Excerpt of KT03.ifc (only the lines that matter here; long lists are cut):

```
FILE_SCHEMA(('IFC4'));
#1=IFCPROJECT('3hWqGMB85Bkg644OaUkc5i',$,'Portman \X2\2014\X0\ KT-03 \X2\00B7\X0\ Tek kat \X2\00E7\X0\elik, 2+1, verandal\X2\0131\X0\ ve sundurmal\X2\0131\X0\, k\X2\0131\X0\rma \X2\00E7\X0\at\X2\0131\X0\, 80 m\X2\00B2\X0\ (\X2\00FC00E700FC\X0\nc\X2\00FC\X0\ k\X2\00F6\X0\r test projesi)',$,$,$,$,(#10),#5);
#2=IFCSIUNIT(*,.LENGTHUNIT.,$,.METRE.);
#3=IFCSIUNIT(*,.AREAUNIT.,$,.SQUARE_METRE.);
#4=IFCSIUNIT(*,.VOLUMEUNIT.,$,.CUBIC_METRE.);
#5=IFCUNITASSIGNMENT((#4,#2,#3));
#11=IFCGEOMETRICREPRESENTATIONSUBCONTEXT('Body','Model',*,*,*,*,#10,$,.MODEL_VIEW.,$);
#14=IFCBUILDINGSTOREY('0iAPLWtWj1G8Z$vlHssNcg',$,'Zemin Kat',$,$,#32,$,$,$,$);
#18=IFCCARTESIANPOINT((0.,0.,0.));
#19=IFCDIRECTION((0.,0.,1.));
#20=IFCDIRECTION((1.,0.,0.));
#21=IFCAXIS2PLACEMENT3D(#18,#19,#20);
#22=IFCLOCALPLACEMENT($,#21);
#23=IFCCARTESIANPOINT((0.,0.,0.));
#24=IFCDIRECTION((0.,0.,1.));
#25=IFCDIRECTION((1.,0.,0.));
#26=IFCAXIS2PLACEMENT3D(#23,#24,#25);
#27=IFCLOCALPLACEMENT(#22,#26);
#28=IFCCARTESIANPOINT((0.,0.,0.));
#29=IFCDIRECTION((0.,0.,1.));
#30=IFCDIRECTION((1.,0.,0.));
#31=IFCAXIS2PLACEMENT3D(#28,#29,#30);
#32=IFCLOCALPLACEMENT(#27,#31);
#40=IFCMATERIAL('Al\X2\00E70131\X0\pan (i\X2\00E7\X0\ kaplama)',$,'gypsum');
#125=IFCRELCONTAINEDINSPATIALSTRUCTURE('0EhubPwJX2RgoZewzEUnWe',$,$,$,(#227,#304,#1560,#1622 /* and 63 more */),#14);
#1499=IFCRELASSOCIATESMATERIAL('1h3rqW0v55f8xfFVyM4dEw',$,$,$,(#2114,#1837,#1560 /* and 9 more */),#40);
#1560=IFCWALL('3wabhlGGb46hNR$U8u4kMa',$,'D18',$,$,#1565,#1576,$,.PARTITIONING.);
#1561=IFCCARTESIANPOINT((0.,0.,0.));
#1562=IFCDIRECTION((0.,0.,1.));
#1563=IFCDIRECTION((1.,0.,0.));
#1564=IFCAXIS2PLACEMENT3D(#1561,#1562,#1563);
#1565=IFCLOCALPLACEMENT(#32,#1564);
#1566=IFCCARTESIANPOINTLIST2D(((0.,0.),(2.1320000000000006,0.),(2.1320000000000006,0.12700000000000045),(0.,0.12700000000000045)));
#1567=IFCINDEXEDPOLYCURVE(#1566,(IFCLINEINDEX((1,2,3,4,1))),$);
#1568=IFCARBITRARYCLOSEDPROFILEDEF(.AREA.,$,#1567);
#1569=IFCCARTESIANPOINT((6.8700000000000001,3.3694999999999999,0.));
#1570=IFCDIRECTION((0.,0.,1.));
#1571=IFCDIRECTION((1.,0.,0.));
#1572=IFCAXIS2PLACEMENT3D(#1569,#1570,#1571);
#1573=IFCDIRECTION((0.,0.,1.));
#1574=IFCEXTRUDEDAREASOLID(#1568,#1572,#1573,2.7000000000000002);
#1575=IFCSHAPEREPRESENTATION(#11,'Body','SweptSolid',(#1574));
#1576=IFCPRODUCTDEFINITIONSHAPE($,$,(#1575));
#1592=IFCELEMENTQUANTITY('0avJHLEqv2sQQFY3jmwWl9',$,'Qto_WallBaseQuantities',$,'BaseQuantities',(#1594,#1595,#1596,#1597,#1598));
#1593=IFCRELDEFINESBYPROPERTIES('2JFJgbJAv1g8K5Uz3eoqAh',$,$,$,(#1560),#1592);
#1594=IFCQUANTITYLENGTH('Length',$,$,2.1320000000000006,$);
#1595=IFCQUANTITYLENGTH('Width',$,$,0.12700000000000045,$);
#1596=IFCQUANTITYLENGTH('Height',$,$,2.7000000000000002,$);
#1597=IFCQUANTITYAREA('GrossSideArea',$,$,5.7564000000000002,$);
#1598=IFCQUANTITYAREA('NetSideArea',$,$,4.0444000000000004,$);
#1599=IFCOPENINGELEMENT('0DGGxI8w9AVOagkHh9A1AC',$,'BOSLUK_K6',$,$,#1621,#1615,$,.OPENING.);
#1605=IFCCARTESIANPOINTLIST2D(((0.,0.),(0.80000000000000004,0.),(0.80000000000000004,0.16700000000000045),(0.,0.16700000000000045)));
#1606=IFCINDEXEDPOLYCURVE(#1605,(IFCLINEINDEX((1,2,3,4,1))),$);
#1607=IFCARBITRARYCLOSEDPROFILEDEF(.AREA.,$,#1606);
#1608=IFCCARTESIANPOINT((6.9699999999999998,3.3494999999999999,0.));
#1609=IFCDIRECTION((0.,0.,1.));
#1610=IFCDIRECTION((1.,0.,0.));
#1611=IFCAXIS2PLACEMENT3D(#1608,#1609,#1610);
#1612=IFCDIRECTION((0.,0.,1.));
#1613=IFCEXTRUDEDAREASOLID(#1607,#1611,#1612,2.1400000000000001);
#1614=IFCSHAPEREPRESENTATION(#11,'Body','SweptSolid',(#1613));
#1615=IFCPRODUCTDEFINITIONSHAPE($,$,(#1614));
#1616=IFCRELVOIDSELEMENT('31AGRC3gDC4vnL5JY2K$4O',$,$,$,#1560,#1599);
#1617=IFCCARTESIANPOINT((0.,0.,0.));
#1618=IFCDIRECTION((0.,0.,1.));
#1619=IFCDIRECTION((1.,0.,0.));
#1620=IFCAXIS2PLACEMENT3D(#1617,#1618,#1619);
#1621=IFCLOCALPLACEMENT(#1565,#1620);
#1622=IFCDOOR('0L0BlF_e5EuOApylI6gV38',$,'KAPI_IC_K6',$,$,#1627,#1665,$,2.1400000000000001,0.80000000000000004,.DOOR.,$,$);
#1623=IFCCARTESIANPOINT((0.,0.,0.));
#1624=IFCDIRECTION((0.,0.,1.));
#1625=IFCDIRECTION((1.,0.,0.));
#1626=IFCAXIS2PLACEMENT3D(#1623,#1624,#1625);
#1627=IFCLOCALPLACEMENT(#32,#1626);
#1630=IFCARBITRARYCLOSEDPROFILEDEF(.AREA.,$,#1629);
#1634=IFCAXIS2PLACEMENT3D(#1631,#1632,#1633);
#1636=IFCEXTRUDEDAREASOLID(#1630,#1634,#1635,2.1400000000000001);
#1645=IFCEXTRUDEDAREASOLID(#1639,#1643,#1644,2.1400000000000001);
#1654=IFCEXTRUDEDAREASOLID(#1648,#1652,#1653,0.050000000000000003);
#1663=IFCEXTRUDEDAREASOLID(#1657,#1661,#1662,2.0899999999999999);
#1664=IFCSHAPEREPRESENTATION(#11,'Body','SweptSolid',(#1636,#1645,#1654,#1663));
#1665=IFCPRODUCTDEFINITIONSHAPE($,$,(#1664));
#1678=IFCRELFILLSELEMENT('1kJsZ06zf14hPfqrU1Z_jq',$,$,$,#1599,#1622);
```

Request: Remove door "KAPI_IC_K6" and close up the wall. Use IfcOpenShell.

```python
import ifcopenshell
import ifcopenshell.api.feature
import ifcopenshell.api.pset
import ifcopenshell.api.root
import ifcopenshell.geom
import ifcopenshell.util.element
import ifcopenshell.util.shape
import ifcopenshell.util.unit

model = ifcopenshell.open("KT03.ifc")
area_scale = ifcopenshell.util.unit.calculate_unit_scale(model, "AREAUNIT")
settings = ifcopenshell.geom.settings()


def volume(element):
    """Net volume in cubic metres, openings subtracted."""
    shape = ifcopenshell.geom.create_shape(settings, element)
    return ifcopenshell.util.shape.get_volume(shape.geometry)


door = model.by_guid("0L0BlF_e5EuOApylI6gV38")
opening = door.FillsVoids[0].RelatingOpeningElement
wall = opening.VoidsElements[0].RelatingBuildingElement
before = volume(wall)

ifcopenshell.api.root.remove_product(model, product=door)
ifcopenshell.api.feature.remove_feature(model, feature=opening)

after = volume(wall)
thickness = 0.127  # wall thickness in metres

# Update the wall's stored quantities.
qto = model.by_id(ifcopenshell.util.element.get_pset(wall, "Qto_WallBaseQuantities", should_inherit=False)["id"])
ifcopenshell.api.pset.edit_qto(model, qto=qto, properties={"NetSideArea": after / thickness / area_scale})

print(f"wall volume {before:.3f} -> {after:.3f} m3")

model.write("KT03_updated.ifc")
```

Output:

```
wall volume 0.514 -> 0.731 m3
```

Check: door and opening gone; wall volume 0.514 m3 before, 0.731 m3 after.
